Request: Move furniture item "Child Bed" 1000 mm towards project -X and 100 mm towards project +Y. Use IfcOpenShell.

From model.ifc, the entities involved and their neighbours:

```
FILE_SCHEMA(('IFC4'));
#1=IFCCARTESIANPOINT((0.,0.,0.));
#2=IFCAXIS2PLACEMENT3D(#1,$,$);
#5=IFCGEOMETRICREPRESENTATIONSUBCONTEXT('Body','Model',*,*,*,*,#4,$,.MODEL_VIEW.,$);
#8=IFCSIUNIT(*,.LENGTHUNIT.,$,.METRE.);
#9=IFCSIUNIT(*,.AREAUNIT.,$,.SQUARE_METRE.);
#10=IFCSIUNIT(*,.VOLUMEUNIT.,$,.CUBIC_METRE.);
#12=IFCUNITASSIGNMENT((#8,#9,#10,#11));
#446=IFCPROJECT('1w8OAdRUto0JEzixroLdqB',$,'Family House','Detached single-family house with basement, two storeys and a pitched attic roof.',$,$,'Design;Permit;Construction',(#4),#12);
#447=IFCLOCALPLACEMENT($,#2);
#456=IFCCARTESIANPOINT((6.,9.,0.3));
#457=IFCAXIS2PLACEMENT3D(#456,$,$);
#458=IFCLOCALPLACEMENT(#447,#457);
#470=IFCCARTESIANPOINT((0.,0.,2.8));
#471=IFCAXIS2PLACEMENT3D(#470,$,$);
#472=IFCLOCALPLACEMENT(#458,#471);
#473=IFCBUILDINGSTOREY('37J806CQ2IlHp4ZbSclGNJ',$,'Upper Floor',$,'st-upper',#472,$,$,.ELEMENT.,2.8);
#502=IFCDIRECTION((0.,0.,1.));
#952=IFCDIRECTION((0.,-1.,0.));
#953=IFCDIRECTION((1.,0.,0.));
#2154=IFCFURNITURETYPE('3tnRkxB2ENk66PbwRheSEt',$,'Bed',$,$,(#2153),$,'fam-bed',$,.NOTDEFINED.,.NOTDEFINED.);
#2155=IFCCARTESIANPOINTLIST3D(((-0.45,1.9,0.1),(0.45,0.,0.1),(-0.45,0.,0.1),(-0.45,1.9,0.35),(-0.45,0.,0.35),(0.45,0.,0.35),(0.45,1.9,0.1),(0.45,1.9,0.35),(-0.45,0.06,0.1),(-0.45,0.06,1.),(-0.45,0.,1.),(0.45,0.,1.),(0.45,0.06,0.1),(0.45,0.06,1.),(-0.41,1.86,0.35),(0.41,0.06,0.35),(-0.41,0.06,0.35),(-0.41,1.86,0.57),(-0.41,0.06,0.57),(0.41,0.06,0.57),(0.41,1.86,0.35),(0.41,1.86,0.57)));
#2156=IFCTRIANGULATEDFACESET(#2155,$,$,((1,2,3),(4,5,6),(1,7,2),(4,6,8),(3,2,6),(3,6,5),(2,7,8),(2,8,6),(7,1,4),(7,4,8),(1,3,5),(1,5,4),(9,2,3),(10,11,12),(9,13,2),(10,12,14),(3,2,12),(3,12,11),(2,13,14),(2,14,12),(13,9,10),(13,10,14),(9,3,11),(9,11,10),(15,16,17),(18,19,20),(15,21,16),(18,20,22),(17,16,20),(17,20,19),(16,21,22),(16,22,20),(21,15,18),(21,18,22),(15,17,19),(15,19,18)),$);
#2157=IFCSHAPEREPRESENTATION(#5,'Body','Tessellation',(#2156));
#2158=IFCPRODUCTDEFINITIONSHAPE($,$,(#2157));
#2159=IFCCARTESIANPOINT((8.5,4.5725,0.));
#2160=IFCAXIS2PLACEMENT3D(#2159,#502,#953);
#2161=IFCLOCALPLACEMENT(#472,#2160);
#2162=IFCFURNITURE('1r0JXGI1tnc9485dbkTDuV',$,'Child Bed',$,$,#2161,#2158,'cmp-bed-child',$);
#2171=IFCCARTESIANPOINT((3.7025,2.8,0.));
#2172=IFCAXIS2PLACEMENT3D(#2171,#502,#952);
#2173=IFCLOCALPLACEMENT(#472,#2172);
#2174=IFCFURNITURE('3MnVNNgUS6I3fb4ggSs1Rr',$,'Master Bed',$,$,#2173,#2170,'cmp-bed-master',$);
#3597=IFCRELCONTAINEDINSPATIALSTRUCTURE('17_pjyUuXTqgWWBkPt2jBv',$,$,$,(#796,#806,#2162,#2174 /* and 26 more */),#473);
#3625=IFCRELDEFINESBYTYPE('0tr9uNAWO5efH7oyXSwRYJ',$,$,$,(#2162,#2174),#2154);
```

```python
import ifcopenshell
import ifcopenshell.api.geometry
import ifcopenshell.util.placement

model = ifcopenshell.open("model.ifc")

item = model.by_guid("1r0JXGI1tnc9485dbkTDuV")
matrix = ifcopenshell.util.placement.get_local_placement(item.ObjectPlacement)
matrix[0, 3] -= 1.0
matrix[1, 3] += 0.1
ifcopenshell.api.geometry.edit_object_placement(model, product=item, matrix=matrix, is_si=False)

print(ifcopenshell.util.placement.get_local_placement(item.ObjectPlacement).round(3) + 0.0)

model.write("model_edited.ifc")
```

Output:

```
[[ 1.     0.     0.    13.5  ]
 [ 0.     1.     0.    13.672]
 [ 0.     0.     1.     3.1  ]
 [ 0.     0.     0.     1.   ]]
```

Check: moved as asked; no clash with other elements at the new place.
